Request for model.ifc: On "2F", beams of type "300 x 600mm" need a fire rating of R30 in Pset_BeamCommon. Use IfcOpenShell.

First a look at what the model holds.

```python
import ifcopenshell
import ifcopenshell.util.element

model = ifcopenshell.open("model.ifc")
print(model.schema)
storey = next(s for s in model.by_type("IfcBuildingStorey") if s.Name == "2F")
beams = [e for e in ifcopenshell.util.element.get_decomposition(storey) if e.is_a("IfcBeam")]
seen = {}
for e in beams:
    element_type = ifcopenshell.util.element.get_type(e)
    key = (element_type.Name if element_type != e and element_type else None, ifcopenshell.util.element.get_pset(e, "Pset_BeamCommon", "FireRating"))
    seen[key] = seen.get(key, 0) + 1
for (name, value), count in sorted(seen.items(), key=str):
    print(count, "x", name, "|", value)
```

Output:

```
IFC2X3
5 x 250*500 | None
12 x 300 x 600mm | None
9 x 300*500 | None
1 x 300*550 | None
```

```python
import ifcopenshell
import ifcopenshell.api.pset
import ifcopenshell.util.element

model = ifcopenshell.open("model.ifc")

storey = next(s for s in model.by_type("IfcBuildingStorey") if s.Name == "2F")
beams = [e for e in ifcopenshell.util.element.get_decomposition(storey) if e.is_a("IfcBeam")]

count = 0
for e in beams:
    element_type = ifcopenshell.util.element.get_type(e)
    if element_type in (None, e) or element_type.Name != "300 x 600mm":
        continue
    # add_pset returns the element's existing set when there is one.
    pset = ifcopenshell.api.pset.add_pset(model, product=e, name="Pset_BeamCommon")
    ifcopenshell.api.pset.edit_pset(model, pset=pset, properties={"FireRating": "R30"})
    count += 1

print(count, "beams updated")

model.write("model-out.ifc")
```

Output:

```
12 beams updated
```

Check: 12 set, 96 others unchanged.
